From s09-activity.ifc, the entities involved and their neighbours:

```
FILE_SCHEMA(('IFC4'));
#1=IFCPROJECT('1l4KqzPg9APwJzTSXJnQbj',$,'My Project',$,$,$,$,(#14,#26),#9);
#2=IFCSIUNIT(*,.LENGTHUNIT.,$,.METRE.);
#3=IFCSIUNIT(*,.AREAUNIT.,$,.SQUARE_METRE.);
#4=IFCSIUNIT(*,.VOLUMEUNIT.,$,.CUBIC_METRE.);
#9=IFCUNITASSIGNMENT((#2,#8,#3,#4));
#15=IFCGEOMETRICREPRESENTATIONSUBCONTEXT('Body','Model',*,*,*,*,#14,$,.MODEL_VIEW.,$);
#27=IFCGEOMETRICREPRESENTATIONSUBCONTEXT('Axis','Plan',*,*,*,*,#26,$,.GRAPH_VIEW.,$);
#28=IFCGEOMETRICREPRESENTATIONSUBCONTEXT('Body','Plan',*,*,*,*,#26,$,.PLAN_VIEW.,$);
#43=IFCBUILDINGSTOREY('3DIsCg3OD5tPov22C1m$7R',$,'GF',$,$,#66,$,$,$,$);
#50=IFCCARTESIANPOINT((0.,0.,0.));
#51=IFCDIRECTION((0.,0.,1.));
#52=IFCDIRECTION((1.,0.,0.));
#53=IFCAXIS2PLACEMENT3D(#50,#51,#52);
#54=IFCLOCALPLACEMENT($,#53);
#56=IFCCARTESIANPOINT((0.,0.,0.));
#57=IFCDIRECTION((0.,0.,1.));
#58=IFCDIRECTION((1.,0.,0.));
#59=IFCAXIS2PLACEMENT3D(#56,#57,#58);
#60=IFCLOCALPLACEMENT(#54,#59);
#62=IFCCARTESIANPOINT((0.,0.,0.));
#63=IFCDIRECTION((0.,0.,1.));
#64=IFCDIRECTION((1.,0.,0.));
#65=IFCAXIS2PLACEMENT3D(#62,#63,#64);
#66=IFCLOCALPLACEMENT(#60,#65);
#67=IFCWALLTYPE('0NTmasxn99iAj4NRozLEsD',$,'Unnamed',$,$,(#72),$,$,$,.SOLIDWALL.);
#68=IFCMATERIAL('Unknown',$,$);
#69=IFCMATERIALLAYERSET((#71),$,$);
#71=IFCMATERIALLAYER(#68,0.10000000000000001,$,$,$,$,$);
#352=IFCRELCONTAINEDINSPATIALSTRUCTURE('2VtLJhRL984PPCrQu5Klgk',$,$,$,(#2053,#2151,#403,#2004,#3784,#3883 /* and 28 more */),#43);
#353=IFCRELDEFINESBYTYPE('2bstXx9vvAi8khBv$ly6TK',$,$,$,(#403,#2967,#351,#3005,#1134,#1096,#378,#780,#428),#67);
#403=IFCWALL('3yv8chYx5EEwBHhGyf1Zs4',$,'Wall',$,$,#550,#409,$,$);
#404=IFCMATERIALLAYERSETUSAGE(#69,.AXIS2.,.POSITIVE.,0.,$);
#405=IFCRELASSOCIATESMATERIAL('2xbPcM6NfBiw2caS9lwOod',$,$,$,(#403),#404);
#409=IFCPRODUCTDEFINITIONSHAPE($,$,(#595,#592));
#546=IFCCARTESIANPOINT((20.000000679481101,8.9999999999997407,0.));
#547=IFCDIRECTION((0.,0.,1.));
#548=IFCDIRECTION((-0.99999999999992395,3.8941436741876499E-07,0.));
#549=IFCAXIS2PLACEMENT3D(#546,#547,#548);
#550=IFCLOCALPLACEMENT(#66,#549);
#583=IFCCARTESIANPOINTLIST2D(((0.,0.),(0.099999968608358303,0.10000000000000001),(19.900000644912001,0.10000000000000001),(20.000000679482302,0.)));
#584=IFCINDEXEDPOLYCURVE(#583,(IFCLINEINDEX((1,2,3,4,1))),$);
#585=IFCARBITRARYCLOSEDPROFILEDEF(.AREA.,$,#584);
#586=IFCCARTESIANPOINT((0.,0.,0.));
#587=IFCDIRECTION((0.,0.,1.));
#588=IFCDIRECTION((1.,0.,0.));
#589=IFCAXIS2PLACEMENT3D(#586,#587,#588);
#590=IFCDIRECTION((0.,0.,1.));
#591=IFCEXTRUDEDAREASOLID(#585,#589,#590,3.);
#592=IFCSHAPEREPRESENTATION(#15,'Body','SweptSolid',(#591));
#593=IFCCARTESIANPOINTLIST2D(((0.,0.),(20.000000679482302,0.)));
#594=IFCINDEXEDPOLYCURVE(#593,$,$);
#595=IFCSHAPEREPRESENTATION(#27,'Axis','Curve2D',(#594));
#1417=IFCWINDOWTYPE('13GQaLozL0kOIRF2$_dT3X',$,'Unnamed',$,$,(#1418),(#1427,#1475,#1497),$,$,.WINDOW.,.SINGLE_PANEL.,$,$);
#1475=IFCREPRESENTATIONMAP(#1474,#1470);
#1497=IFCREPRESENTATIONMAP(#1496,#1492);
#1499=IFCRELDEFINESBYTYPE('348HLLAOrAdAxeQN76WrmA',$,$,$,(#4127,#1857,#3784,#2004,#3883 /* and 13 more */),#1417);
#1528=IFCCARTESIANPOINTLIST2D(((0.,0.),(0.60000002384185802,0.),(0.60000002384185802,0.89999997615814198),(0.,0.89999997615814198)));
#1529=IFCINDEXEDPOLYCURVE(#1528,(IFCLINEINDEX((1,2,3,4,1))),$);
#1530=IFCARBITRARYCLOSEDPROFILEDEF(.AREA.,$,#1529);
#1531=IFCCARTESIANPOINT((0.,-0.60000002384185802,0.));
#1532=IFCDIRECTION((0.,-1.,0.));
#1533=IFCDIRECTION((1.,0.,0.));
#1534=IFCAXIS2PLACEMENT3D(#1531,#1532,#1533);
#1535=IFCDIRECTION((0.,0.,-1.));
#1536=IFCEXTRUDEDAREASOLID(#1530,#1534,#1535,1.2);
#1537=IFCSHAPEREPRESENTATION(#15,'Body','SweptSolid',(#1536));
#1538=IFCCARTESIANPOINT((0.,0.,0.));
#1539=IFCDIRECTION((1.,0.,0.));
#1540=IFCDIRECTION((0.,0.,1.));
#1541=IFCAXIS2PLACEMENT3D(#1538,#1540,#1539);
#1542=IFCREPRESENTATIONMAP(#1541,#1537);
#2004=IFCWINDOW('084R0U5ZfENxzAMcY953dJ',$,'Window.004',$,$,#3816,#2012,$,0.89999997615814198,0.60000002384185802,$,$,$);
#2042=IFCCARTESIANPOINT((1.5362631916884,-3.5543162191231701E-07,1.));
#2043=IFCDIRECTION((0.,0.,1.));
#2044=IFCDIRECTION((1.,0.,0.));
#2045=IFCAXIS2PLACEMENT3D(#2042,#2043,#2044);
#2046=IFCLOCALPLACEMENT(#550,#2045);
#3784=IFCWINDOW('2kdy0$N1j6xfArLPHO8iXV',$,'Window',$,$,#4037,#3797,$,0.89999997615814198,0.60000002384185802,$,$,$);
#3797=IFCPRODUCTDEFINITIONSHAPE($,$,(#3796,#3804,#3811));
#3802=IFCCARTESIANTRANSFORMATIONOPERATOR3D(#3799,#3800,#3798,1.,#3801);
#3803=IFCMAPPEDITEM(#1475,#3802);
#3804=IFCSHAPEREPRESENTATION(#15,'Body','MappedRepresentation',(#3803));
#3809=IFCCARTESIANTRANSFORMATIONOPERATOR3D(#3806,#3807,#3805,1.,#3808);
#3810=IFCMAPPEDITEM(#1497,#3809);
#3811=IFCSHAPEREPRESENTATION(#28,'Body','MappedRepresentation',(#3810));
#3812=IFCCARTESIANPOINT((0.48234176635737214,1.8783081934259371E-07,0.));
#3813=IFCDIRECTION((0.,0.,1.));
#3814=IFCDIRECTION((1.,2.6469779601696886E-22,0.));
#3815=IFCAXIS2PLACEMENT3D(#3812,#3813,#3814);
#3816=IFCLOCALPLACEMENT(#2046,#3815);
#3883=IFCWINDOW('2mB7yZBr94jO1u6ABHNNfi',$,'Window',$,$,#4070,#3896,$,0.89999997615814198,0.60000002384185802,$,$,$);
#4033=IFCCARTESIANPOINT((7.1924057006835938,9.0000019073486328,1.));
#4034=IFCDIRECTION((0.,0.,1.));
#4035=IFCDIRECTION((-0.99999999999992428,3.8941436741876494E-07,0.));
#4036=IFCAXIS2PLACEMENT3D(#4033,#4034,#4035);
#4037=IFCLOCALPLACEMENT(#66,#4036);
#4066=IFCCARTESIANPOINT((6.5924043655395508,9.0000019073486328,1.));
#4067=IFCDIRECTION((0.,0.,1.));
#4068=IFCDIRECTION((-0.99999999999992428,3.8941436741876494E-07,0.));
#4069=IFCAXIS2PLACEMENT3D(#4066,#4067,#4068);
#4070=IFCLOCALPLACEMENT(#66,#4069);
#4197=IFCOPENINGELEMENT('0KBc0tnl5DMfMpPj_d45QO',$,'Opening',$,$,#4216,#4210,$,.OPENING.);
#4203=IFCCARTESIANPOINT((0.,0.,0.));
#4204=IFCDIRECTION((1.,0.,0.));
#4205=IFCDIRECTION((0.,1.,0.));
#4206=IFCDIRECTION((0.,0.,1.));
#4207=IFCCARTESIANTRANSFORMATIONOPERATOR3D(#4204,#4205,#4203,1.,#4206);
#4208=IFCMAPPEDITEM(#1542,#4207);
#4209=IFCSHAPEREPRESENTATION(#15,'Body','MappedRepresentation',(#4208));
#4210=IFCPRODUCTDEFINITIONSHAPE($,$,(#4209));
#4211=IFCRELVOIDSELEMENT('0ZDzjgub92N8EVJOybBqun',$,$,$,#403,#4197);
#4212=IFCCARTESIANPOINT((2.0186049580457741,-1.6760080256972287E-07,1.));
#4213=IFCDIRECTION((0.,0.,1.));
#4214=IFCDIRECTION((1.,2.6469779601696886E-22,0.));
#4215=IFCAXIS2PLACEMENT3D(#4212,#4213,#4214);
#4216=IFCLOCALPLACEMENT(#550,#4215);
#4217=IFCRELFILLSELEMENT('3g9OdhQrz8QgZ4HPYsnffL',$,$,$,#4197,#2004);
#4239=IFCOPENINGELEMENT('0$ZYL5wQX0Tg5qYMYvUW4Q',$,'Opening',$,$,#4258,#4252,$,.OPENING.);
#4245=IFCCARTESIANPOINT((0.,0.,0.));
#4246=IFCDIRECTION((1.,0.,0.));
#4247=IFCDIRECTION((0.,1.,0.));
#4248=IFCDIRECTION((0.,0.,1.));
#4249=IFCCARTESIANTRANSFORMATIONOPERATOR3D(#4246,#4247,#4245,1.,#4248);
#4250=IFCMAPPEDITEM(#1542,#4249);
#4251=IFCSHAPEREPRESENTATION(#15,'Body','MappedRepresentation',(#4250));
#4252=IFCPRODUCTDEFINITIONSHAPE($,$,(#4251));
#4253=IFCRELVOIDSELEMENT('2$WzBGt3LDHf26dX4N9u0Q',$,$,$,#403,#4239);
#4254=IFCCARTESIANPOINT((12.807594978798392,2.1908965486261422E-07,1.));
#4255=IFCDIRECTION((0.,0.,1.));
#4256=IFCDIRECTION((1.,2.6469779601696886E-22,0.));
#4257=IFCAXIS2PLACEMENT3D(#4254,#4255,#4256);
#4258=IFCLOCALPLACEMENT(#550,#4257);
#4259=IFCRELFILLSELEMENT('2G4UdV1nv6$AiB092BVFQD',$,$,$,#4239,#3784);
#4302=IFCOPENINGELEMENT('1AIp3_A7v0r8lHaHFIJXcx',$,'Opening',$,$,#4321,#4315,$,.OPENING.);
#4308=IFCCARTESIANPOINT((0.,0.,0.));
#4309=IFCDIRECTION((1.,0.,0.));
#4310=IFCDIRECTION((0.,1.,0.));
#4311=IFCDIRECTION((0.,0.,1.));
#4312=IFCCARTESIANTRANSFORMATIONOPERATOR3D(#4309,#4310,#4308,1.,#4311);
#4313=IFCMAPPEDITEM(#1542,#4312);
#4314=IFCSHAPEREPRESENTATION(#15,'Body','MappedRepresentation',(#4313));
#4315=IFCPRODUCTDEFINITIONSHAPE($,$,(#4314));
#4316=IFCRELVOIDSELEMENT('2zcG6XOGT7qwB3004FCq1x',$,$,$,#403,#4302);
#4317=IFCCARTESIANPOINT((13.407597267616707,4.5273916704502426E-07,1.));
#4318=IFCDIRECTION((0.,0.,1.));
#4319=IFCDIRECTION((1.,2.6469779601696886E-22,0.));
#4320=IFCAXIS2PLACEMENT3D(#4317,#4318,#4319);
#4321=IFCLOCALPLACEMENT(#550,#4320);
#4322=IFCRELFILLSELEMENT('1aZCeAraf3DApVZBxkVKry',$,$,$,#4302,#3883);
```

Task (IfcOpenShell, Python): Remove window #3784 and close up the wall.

```python
import ifcopenshell
import ifcopenshell.api.feature
import ifcopenshell.api.root
import ifcopenshell.geom
import ifcopenshell.util.shape

model = ifcopenshell.open("s09-activity.ifc")
settings = ifcopenshell.geom.settings()


def volume(element):
    """Net volume in cubic metres, openings subtracted."""
    shape = ifcopenshell.geom.create_shape(settings, element)
    return ifcopenshell.util.shape.get_volume(shape.geometry)


window = model.by_guid("2kdy0$N1j6xfArLPHO8iXV")
opening = window.FillsVoids[0].RelatingOpeningElement
wall = opening.VoidsElements[0].RelatingBuildingElement
before = volume(wall)

ifcopenshell.api.root.remove_product(model, product=window)
ifcopenshell.api.feature.remove_feature(model, feature=opening)

after = volume(wall)

print(f"wall volume {before:.3f} -> {after:.3f} m3")

model.write("s09-activity_updated.ifc")
```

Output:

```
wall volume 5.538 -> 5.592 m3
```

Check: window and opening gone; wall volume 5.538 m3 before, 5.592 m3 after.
